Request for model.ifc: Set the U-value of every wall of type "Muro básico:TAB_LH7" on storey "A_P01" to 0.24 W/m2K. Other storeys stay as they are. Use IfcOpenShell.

First a look at what the model holds.

```python
import ifcopenshell
import ifcopenshell.util.element

model = ifcopenshell.open("model.ifc")
print(model.schema)
storey = next(s for s in model.by_type("IfcBuildingStorey") if s.Name == "A_P01")
walls = [e for e in ifcopenshell.util.element.get_decomposition(storey) if e.is_a("IfcWall")]
seen = {}
for e in walls:
    element_type = ifcopenshell.util.element.get_type(e)
    key = (element_type.Name if element_type != e and element_type else None, ifcopenshell.util.element.get_pset(e, "Pset_WallCommon", "ThermalTransmittance"))
    seen[key] = seen.get(key, 0) + 1
for (name, value), count in sorted(seen.items(), key=str):
    print(count, "x", name, "|", value)
```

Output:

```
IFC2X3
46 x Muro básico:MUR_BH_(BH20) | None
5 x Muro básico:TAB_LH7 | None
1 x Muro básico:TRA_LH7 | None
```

```python
import ifcopenshell
import ifcopenshell.api.pset
import ifcopenshell.util.element

model = ifcopenshell.open("model.ifc")

storey = next(s for s in model.by_type("IfcBuildingStorey") if s.Name == "A_P01")
walls = [e for e in ifcopenshell.util.element.get_decomposition(storey) if e.is_a("IfcWall")]

count = 0
for e in walls:
    element_type = ifcopenshell.util.element.get_type(e)
    if element_type in (None, e) or element_type.Name != "Muro básico:TAB_LH7":
        continue
    # add_pset returns the element's existing set when there is one.
    pset = ifcopenshell.api.pset.add_pset(model, product=e, name="Pset_WallCommon")
    ifcopenshell.api.pset.edit_pset(model, pset=pset, properties={"ThermalTransmittance": 0.24})
    count += 1

print(count, "walls updated")

model.write("model_v2.ifc")
```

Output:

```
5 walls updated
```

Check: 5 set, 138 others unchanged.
